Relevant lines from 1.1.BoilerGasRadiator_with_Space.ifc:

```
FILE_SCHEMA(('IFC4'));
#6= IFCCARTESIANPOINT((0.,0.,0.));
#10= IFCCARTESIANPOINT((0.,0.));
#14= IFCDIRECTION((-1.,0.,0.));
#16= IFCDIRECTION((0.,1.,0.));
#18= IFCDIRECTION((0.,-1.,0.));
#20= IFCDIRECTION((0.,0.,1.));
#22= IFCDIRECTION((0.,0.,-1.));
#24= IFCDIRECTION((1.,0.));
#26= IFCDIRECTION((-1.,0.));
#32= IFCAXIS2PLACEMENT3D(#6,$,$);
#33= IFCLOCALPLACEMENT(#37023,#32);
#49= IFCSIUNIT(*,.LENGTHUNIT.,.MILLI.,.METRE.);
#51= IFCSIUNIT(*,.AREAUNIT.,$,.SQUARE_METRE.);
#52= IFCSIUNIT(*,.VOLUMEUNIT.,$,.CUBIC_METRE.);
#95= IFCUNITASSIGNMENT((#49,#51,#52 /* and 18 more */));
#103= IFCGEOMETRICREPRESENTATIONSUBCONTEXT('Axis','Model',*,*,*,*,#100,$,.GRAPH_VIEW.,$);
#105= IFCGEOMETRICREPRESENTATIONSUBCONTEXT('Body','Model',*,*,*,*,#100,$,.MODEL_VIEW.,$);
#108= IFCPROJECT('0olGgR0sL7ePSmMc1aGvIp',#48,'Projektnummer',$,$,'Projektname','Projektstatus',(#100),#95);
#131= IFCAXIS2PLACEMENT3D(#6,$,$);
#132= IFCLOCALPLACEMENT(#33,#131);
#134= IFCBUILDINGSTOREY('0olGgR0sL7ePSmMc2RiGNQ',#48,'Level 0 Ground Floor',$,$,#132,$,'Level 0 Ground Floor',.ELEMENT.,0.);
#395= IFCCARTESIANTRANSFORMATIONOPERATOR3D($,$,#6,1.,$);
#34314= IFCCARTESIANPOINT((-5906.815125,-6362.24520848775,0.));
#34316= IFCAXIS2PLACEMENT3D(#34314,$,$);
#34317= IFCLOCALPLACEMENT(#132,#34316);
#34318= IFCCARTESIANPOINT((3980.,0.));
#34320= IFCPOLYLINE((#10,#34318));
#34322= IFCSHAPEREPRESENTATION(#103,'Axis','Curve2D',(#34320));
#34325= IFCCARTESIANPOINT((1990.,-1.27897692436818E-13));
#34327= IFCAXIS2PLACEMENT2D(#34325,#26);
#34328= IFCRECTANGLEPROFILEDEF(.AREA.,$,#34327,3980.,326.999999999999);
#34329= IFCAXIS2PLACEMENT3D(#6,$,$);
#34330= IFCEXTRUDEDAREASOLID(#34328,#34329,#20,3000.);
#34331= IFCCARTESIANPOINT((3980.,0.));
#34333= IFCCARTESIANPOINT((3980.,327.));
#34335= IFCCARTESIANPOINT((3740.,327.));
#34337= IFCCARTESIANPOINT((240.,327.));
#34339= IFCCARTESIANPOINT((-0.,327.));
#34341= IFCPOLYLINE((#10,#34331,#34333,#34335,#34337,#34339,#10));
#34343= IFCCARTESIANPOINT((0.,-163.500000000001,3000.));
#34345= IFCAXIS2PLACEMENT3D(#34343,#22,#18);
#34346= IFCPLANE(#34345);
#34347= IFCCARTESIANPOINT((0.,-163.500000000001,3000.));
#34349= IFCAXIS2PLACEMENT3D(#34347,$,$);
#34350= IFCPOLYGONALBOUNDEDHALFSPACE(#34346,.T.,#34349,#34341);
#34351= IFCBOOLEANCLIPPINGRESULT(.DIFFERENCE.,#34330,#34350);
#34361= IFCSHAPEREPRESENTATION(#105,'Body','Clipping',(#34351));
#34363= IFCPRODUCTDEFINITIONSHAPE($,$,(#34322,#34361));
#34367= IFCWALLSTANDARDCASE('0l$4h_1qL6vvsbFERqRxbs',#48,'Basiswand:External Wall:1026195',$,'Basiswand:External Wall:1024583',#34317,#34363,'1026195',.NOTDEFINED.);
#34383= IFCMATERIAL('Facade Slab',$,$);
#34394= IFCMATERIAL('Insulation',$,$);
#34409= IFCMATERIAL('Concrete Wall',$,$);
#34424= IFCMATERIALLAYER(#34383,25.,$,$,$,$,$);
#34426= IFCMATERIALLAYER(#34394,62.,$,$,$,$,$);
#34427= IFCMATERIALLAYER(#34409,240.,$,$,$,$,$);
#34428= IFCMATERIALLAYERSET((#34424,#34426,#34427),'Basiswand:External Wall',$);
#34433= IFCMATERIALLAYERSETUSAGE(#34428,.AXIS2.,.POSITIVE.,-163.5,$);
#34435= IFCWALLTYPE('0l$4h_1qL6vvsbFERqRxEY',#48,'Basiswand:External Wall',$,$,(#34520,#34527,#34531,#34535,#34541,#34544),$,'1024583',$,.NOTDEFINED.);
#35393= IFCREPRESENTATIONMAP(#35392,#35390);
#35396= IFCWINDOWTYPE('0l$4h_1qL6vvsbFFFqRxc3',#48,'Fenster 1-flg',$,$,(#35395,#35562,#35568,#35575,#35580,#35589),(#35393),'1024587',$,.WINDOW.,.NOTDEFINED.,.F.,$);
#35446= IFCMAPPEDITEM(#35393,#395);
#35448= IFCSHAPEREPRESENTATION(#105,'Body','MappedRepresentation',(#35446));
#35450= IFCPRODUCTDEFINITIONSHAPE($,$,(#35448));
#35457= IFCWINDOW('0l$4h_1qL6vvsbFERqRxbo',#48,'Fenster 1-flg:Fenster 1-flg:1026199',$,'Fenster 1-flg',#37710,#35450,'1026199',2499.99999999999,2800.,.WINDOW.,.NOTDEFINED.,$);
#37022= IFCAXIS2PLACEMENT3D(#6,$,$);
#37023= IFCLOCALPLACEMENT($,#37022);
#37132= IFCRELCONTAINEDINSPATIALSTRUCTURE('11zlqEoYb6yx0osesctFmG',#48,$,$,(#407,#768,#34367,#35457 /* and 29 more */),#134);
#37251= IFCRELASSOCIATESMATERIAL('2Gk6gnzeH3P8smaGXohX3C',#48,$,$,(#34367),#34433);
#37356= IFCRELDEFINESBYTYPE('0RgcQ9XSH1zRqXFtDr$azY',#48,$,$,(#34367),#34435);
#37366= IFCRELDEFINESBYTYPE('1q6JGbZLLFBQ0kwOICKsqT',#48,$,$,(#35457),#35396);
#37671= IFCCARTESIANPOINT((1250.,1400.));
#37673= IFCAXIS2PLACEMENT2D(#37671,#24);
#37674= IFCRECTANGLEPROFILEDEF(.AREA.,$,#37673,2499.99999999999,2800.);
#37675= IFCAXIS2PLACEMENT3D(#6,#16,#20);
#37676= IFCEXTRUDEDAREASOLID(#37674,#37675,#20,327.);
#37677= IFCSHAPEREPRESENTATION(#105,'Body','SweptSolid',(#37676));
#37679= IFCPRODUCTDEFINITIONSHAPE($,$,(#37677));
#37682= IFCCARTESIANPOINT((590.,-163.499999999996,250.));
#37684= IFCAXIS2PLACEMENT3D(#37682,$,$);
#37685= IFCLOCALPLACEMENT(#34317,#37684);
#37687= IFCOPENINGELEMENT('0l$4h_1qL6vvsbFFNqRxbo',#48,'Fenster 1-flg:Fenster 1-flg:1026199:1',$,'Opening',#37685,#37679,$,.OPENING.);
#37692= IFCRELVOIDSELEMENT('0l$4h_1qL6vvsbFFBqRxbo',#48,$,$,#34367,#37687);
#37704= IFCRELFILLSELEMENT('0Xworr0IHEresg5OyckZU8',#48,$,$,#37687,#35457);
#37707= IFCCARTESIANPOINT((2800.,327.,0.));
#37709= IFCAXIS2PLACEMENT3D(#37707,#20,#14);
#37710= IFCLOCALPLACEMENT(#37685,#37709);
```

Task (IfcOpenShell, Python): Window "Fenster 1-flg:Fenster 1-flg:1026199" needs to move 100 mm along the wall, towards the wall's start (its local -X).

```python
import ifcopenshell
import ifcopenshell.api.geometry
import ifcopenshell.util.placement
import ifcopenshell.util.unit

model = ifcopenshell.open("1.1.BoilerGasRadiator_with_Space.ifc")
unit_scale = ifcopenshell.util.unit.calculate_unit_scale(model)

window = model.by_id(35457)
opening = window.FillsVoids[0].RelatingOpeningElement
wall = opening.VoidsElements[0].RelatingBuildingElement

wall_matrix = ifcopenshell.util.placement.get_local_placement(wall.ObjectPlacement)
shift = wall_matrix[:3, 0] * -0.1 / unit_scale
before = ifcopenshell.util.placement.get_local_placement(window.ObjectPlacement)[:3, 3].copy()

# The window is placed relative to its opening, so it follows when the opening moves.
matrix = ifcopenshell.util.placement.get_local_placement(opening.ObjectPlacement)
matrix[:3, 3] += shift
ifcopenshell.api.geometry.edit_object_placement(
    model, product=opening, matrix=matrix, is_si=False, should_transform_children=True
)

after = ifcopenshell.util.placement.get_local_placement(window.ObjectPlacement)[:3, 3]
print("window moved by", (after - before).round(3) + 0.0)

model.write("1.1.BoilerGasRadiator_with_Space_edited.ifc")
```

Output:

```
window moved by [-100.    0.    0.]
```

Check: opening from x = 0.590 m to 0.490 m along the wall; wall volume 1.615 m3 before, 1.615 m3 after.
